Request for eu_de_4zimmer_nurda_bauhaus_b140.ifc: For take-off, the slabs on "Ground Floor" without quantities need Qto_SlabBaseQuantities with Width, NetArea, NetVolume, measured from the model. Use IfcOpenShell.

First a look at what the model holds.

```python
import ifcopenshell
import ifcopenshell.util.element
import ifcopenshell.util.unit

model = ifcopenshell.open("eu_de_4zimmer_nurda_bauhaus_b140.ifc")
print(model.schema)
for unit_type in ("LENGTHUNIT", "AREAUNIT", "VOLUMEUNIT"):
    print(unit_type, ifcopenshell.util.unit.calculate_unit_scale(model, unit_type))
storey = next(s for s in model.by_type("IfcBuildingStorey") if s.Name == "Ground Floor")
slabs = [e for e in ifcopenshell.util.element.get_decomposition(storey) if e.is_a("IfcSlab")]
for e in sorted(slabs, key=lambda e: e.id()):
    print(e.id(), e.is_a(), e.Name, list(ifcopenshell.util.element.get_psets(e, qtos_only=True)), sep=" | ")
```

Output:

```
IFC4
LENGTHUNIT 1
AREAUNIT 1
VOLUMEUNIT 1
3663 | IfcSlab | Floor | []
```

```python
import ifcopenshell
import ifcopenshell.api.pset
import ifcopenshell.geom
import ifcopenshell.util.element
import ifcopenshell.util.shape
import ifcopenshell.util.unit

model = ifcopenshell.open("eu_de_4zimmer_nurda_bauhaus_b140.ifc")
unit_scale = ifcopenshell.util.unit.calculate_unit_scale(model)
area_scale = ifcopenshell.util.unit.calculate_unit_scale(model, "AREAUNIT")
volume_scale = ifcopenshell.util.unit.calculate_unit_scale(model, "VOLUMEUNIT")
settings = ifcopenshell.geom.settings()

storey = next(s for s in model.by_type("IfcBuildingStorey") if s.Name == "Ground Floor")
slabs = [e for e in ifcopenshell.util.element.get_decomposition(storey) if e.is_a("IfcSlab")]

for e in sorted(slabs, key=lambda e: e.id()):
    if ifcopenshell.util.element.get_psets(e, qtos_only=True, should_inherit=False):
        continue
    # Geometry comes back in metres, in the element's own axes.
    shape = ifcopenshell.geom.create_shape(settings, e)
    values = {
        "Width": ifcopenshell.util.shape.get_z(shape.geometry) / unit_scale,
        "NetArea": ifcopenshell.util.shape.get_footprint_area(shape.geometry) / area_scale,
        "NetVolume": ifcopenshell.util.shape.get_volume(shape.geometry) / volume_scale,
    }
    qto = ifcopenshell.api.pset.add_qto(model, product=e, name="Qto_SlabBaseQuantities")
    ifcopenshell.api.pset.edit_qto(model, qto=qto, properties=values)
    print(e.id(), {k: round(v, 3) for k, v in values.items()})

model.write("eu_de_4zimmer_nurda_bauhaus_b140-out.ifc")
```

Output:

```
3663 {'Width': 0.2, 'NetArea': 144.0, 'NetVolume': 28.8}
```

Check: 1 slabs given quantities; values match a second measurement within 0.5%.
